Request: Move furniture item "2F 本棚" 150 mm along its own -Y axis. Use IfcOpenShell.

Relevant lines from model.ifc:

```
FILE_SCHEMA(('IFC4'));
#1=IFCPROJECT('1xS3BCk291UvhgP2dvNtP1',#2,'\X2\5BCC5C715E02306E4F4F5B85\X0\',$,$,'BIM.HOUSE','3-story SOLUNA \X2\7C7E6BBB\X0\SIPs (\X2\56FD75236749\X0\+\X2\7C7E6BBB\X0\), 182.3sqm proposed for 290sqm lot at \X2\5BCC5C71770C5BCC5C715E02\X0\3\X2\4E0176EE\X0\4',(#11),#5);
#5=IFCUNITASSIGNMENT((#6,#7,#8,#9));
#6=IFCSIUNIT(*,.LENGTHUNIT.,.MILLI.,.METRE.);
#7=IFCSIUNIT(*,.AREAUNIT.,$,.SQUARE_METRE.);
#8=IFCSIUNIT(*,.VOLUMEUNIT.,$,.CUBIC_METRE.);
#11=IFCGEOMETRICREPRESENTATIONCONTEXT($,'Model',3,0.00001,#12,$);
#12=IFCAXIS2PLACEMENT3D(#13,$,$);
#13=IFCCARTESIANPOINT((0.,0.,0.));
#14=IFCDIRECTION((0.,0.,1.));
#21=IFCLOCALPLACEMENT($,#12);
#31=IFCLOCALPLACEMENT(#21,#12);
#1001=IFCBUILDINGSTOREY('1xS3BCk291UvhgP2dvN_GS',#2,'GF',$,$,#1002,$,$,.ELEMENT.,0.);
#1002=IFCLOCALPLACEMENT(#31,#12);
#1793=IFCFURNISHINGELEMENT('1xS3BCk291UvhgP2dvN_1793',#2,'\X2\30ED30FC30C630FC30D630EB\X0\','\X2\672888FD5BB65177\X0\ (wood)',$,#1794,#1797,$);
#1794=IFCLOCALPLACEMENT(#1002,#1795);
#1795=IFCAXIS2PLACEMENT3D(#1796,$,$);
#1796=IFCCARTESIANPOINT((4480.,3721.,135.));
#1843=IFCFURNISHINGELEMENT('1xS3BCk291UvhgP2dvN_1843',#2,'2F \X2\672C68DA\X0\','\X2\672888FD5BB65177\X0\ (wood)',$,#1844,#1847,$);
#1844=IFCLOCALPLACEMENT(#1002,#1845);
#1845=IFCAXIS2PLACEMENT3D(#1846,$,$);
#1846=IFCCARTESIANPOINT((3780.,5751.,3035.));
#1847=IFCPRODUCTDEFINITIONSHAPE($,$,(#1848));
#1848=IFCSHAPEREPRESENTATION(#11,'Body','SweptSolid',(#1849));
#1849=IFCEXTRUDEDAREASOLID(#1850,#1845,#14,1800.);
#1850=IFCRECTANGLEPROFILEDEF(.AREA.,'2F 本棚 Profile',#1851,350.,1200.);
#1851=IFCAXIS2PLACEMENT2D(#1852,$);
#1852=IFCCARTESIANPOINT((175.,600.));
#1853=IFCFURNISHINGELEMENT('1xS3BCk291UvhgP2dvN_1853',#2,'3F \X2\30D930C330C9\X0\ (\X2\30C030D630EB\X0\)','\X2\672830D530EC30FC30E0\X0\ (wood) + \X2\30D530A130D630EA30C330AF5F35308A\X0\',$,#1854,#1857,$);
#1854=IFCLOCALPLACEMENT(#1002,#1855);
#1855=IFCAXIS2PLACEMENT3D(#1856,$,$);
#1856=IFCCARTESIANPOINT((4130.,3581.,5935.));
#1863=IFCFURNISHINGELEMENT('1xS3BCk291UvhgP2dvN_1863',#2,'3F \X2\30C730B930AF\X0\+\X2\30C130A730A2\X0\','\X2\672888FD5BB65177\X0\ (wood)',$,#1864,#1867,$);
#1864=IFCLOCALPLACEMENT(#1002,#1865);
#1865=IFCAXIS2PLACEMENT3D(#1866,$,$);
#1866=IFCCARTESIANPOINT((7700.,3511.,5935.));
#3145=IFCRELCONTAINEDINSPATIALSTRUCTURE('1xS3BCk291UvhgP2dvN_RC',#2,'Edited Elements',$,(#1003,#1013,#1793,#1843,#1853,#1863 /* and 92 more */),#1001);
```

```python
import ifcopenshell
import ifcopenshell.api.geometry
import ifcopenshell.util.placement
import ifcopenshell.util.unit

model = ifcopenshell.open("model.ifc")
unit_scale = ifcopenshell.util.unit.calculate_unit_scale(model)

item = model.by_guid("1xS3BCk291UvhgP2dvN_1843")
matrix = ifcopenshell.util.placement.get_local_placement(item.ObjectPlacement)
matrix[:3, 3] -= matrix[:3, 1] * 0.15 / unit_scale
ifcopenshell.api.geometry.edit_object_placement(model, product=item, matrix=matrix, is_si=False)

print(ifcopenshell.util.placement.get_local_placement(item.ObjectPlacement).round(3) + 0.0)

model.write("model-out.ifc")
```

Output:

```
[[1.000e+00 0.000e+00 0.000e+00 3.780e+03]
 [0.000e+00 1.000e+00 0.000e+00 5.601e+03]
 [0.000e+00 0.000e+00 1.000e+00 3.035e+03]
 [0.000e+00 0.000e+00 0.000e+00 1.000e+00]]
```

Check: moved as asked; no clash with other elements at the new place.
